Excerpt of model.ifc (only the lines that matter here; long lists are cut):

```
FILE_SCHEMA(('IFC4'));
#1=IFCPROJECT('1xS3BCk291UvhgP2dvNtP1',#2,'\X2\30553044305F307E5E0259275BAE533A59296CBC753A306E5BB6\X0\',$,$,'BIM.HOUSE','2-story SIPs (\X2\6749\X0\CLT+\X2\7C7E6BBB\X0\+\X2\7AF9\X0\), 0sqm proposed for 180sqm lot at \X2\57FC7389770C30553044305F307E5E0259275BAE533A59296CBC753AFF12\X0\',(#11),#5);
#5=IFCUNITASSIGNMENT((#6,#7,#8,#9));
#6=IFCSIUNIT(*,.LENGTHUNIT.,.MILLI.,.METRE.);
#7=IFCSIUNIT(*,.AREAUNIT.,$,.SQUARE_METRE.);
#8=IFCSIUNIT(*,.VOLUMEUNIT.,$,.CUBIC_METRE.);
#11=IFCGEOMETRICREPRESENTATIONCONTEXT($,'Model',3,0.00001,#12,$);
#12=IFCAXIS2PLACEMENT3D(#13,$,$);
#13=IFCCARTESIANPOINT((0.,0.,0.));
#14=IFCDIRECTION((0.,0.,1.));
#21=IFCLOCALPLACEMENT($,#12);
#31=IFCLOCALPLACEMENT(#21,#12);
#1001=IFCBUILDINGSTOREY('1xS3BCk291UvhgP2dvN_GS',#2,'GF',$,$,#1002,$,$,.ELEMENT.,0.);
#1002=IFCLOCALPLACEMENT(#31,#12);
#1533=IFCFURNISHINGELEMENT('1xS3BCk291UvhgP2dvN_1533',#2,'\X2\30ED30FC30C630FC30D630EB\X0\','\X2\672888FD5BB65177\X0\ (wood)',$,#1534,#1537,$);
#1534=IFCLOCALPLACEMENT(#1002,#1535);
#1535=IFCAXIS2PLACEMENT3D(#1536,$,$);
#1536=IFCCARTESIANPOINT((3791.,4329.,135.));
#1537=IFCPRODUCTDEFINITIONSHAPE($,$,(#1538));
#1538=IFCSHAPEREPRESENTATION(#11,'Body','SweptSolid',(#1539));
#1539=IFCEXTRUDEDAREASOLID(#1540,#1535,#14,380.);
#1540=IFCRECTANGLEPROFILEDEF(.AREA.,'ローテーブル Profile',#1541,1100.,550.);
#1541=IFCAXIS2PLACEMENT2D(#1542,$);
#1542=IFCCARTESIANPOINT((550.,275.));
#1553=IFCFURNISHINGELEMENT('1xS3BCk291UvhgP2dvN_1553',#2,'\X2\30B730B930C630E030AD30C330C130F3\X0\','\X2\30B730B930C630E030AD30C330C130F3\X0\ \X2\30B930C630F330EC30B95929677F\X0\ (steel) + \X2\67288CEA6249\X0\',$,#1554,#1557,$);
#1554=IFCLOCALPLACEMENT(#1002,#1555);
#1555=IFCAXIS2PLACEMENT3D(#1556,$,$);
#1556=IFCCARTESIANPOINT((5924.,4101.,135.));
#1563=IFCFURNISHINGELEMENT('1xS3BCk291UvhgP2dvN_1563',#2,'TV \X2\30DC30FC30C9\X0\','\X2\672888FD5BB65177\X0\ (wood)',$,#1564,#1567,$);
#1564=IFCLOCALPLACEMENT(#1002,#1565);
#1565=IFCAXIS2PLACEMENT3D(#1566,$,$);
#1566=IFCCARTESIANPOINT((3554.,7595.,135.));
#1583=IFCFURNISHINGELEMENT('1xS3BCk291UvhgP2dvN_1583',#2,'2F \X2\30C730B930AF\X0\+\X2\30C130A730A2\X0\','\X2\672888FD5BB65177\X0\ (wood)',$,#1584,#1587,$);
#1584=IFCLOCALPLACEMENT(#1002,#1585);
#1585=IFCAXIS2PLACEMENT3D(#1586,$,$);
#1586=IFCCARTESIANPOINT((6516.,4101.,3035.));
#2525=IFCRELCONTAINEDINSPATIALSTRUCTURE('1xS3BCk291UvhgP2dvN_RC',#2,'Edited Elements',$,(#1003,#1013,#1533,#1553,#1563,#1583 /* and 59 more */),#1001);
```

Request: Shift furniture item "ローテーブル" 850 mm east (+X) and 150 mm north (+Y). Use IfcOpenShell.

```python
import ifcopenshell
import ifcopenshell.api.geometry
import ifcopenshell.util.placement

model = ifcopenshell.open("model.ifc")

item = model.by_id(1533)
matrix = ifcopenshell.util.placement.get_local_placement(item.ObjectPlacement)
matrix[0, 3] += 850.0
matrix[1, 3] += 150.0
ifcopenshell.api.geometry.edit_object_placement(model, product=item, matrix=matrix, is_si=False)

print(ifcopenshell.util.placement.get_local_placement(item.ObjectPlacement).round(3) + 0.0)

model.write("model_edited.ifc")
```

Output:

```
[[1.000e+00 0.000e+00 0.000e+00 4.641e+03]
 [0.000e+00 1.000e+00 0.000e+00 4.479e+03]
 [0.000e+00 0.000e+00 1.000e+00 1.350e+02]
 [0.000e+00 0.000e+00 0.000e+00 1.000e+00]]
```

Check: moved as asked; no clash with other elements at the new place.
